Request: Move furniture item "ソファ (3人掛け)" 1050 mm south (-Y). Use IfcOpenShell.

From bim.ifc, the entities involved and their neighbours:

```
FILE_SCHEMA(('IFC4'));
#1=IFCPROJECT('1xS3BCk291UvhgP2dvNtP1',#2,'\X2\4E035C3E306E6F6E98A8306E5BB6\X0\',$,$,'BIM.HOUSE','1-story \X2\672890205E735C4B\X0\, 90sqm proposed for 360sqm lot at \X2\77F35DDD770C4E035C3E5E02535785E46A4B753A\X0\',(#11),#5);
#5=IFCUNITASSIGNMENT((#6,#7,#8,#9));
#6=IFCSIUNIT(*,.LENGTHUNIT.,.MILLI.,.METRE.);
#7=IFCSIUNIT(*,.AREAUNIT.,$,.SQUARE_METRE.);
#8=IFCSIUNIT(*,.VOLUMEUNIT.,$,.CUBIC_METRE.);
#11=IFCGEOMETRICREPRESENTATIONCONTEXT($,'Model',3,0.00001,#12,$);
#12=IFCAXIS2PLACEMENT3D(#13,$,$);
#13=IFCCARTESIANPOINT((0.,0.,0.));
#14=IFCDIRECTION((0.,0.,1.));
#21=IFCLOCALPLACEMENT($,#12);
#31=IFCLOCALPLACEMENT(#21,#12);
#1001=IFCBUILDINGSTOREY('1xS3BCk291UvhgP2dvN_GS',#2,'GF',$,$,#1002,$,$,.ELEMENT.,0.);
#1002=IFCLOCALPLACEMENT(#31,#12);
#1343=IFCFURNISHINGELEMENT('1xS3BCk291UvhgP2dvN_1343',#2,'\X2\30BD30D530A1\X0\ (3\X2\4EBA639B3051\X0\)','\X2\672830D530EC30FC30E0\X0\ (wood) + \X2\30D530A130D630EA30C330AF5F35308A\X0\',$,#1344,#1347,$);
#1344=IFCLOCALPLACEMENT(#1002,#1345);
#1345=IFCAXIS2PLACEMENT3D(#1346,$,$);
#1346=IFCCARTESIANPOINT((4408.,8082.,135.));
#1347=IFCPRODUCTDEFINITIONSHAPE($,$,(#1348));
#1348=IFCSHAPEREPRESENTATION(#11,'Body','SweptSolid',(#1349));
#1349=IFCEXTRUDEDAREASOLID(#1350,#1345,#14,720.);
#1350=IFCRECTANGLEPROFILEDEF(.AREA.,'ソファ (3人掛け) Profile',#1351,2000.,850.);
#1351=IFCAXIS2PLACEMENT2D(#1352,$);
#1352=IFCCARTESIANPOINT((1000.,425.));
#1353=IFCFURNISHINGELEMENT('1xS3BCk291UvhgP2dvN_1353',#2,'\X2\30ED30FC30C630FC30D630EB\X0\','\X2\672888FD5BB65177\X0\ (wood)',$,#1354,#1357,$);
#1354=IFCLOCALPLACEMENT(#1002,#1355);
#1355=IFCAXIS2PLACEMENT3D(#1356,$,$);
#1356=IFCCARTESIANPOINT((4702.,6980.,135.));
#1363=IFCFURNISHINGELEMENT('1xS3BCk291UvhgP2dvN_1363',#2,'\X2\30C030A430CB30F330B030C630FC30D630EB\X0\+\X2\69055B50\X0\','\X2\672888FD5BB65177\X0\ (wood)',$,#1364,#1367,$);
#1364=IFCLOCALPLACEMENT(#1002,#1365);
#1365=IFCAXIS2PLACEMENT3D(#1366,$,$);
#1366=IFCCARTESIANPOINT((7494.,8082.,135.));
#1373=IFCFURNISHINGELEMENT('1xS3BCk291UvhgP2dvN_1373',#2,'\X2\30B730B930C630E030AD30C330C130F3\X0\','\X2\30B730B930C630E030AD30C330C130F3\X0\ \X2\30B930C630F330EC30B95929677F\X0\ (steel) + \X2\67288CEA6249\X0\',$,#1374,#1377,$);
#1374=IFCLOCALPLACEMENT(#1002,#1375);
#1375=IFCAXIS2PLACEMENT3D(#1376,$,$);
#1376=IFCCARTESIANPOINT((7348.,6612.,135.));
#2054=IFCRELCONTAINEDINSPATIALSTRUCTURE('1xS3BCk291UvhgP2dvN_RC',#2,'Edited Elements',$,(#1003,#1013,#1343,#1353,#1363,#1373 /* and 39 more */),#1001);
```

```python
import ifcopenshell
import ifcopenshell.api.geometry
import ifcopenshell.util.placement

model = ifcopenshell.open("bim.ifc")

item = model.by_id(1343)
matrix = ifcopenshell.util.placement.get_local_placement(item.ObjectPlacement)
matrix[1, 3] -= 1050.0
ifcopenshell.api.geometry.edit_object_placement(model, product=item, matrix=matrix, is_si=False)

print(ifcopenshell.util.placement.get_local_placement(item.ObjectPlacement).round(3) + 0.0)

model.write("bim_edited.ifc")
```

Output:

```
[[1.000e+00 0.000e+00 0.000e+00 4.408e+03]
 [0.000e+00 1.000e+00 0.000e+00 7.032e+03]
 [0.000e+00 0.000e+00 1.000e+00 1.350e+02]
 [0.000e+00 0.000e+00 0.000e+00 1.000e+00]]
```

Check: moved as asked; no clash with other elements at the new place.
